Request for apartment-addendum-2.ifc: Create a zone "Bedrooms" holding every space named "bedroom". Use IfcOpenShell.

First a look at what the model holds.

```python
import ifcopenshell

model = ifcopenshell.open("apartment-addendum-2.ifc")
print(model.schema)
seen = {}
for space in model.by_type("IfcSpace"):
    seen[space.LongName] = seen.get(space.LongName, 0) + 1
for name, count in sorted(seen.items(), key=str):
    print(count, "x", name)
print("zones:", [z.Name for z in model.by_type("IfcZone")][:20])
```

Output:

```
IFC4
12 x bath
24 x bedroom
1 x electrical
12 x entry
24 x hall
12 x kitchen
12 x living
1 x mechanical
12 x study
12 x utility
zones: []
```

```python
import ifcopenshell
import ifcopenshell.api.group
import ifcopenshell.api.root

model = ifcopenshell.open("apartment-addendum-2.ifc")

names = {"bedroom"}
spaces = [s for s in model.by_type("IfcSpace") if s.LongName in names]

zone = ifcopenshell.api.root.create_entity(model, ifc_class="IfcZone", name="Bedrooms")
ifcopenshell.api.group.assign_group(model, products=spaces, group=zone)
print(len(spaces), "spaces in", zone.Name)

model.write("apartment-addendum-2_v2.ifc")
```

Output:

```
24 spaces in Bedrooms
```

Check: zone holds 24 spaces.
